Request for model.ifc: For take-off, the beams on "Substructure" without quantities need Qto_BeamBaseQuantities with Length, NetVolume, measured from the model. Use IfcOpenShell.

First a look at what the model holds.

```python
import ifcopenshell
import ifcopenshell.util.element
import ifcopenshell.util.unit

model = ifcopenshell.open("model.ifc")
print(model.schema)
for unit_type in ("LENGTHUNIT", "AREAUNIT", "VOLUMEUNIT"):
    print(unit_type, ifcopenshell.util.unit.calculate_unit_scale(model, unit_type))
storey = next(s for s in model.by_type("IfcBuildingStorey") if s.Name == "Substructure")
beams = [e for e in ifcopenshell.util.element.get_decomposition(storey) if e.is_a("IfcBeam")]
for e in sorted(beams, key=lambda e: e.id()):
    print(e.id(), e.is_a(), e.Name, list(ifcopenshell.util.element.get_psets(e, qtos_only=True)), sep=" | ")
```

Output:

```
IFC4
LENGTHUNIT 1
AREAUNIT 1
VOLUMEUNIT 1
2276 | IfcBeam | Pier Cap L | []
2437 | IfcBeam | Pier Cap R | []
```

```python
import ifcopenshell
import ifcopenshell.api.pset
import ifcopenshell.geom
import ifcopenshell.util.element
import ifcopenshell.util.shape
import ifcopenshell.util.unit

model = ifcopenshell.open("model.ifc")
unit_scale = ifcopenshell.util.unit.calculate_unit_scale(model)
volume_scale = ifcopenshell.util.unit.calculate_unit_scale(model, "VOLUMEUNIT")
settings = ifcopenshell.geom.settings()

storey = next(s for s in model.by_type("IfcBuildingStorey") if s.Name == "Substructure")
beams = [e for e in ifcopenshell.util.element.get_decomposition(storey) if e.is_a("IfcBeam")]

for e in sorted(beams, key=lambda e: e.id()):
    if ifcopenshell.util.element.get_psets(e, qtos_only=True, should_inherit=False):
        continue
    # Geometry comes back in metres, in the element's own axes.
    shape = ifcopenshell.geom.create_shape(settings, e)
    values = {
        "Length": ifcopenshell.util.shape.get_max_xyz(shape.geometry) / unit_scale,
        "NetVolume": ifcopenshell.util.shape.get_volume(shape.geometry) / volume_scale,
    }
    qto = ifcopenshell.api.pset.add_qto(model, product=e, name="Qto_BeamBaseQuantities")
    ifcopenshell.api.pset.edit_qto(model, qto=qto, properties=values)
    print(e.id(), {k: round(v, 3) for k, v in values.items()})

model.write("model_v2.ifc")
```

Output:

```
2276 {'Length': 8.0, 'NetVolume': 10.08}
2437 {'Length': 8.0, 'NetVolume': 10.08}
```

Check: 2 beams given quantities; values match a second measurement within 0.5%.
